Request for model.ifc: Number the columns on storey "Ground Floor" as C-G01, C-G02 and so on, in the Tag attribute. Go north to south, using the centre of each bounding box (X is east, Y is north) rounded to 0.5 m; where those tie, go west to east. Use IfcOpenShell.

First a look at what the model holds.

```python
import ifcopenshell
import ifcopenshell.util.element
import ifcopenshell.util.placement

model = ifcopenshell.open("model.ifc")
print(model.schema)
storey = next(s for s in model.by_type("IfcBuildingStorey") if s.Name == "Ground Floor")
columns = [e for e in ifcopenshell.util.element.get_decomposition(storey) if e.is_a("IfcColumn")]
for e in sorted(columns, key=lambda e: e.id()):
    origin = ifcopenshell.util.placement.get_local_placement(e.ObjectPlacement)[:3, 3]
    print(e.id(), e.Tag, e.Name, origin.round(2) + 0.0, sep=" | ")
```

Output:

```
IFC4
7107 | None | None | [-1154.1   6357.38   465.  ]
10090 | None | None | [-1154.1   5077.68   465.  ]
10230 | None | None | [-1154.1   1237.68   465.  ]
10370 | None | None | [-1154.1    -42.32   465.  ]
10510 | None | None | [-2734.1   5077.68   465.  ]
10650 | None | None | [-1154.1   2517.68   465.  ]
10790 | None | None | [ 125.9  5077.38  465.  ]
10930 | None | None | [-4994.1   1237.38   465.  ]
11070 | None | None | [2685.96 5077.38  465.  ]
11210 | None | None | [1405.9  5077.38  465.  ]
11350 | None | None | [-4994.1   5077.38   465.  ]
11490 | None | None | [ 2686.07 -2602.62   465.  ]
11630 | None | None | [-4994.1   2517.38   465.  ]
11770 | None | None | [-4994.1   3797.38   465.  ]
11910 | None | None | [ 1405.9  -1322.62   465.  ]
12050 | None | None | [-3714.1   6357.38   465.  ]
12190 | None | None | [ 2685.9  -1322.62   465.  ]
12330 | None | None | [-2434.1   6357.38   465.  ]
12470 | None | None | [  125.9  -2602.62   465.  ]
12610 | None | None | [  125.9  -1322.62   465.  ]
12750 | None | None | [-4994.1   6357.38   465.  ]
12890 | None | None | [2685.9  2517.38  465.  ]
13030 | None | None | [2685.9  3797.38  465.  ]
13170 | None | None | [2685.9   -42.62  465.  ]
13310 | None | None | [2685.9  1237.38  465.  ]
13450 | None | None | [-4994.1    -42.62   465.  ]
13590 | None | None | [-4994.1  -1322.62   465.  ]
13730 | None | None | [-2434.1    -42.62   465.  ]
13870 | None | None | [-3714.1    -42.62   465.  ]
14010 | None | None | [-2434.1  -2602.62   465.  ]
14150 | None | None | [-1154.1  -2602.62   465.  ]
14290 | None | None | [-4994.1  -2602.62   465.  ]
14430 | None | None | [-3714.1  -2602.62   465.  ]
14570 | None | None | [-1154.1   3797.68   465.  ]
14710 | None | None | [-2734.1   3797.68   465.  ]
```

```python
import ifcopenshell
import ifcopenshell.geom
import ifcopenshell.util.element
import ifcopenshell.util.shape

model = ifcopenshell.open("model.ifc")
settings = ifcopenshell.geom.settings()
settings.set("use-world-coords", True)


def centre(element):
    shape = ifcopenshell.geom.create_shape(settings, element)
    return ifcopenshell.util.shape.get_bbox_centroid(shape.geometry)


storey = next(s for s in model.by_type("IfcBuildingStorey") if s.Name == "Ground Floor")
columns = [e for e in ifcopenshell.util.element.get_decomposition(storey) if e.is_a("IfcColumn")]

# Insertion points can sit at a corner or the storey origin, so sort by the geometry (in metres).
centres = {e: centre(e) for e in columns}
columns.sort(key=lambda e: (-round(centres[e][1] / 0.5), centres[e][0]))

for i, e in enumerate(columns, start=1):
    number = f"C-G{i:02d}"
    e.Tag = number
    print(e.id(), number)

model.write("model-out.ifc")
```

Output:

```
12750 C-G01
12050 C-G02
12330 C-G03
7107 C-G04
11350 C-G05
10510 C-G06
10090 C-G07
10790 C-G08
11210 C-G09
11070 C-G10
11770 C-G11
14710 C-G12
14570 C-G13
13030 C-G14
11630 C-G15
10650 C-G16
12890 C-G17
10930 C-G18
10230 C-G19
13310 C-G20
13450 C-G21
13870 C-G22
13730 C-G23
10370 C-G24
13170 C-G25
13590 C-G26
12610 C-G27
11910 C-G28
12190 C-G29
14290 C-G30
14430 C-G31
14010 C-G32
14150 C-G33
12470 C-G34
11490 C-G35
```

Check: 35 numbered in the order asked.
